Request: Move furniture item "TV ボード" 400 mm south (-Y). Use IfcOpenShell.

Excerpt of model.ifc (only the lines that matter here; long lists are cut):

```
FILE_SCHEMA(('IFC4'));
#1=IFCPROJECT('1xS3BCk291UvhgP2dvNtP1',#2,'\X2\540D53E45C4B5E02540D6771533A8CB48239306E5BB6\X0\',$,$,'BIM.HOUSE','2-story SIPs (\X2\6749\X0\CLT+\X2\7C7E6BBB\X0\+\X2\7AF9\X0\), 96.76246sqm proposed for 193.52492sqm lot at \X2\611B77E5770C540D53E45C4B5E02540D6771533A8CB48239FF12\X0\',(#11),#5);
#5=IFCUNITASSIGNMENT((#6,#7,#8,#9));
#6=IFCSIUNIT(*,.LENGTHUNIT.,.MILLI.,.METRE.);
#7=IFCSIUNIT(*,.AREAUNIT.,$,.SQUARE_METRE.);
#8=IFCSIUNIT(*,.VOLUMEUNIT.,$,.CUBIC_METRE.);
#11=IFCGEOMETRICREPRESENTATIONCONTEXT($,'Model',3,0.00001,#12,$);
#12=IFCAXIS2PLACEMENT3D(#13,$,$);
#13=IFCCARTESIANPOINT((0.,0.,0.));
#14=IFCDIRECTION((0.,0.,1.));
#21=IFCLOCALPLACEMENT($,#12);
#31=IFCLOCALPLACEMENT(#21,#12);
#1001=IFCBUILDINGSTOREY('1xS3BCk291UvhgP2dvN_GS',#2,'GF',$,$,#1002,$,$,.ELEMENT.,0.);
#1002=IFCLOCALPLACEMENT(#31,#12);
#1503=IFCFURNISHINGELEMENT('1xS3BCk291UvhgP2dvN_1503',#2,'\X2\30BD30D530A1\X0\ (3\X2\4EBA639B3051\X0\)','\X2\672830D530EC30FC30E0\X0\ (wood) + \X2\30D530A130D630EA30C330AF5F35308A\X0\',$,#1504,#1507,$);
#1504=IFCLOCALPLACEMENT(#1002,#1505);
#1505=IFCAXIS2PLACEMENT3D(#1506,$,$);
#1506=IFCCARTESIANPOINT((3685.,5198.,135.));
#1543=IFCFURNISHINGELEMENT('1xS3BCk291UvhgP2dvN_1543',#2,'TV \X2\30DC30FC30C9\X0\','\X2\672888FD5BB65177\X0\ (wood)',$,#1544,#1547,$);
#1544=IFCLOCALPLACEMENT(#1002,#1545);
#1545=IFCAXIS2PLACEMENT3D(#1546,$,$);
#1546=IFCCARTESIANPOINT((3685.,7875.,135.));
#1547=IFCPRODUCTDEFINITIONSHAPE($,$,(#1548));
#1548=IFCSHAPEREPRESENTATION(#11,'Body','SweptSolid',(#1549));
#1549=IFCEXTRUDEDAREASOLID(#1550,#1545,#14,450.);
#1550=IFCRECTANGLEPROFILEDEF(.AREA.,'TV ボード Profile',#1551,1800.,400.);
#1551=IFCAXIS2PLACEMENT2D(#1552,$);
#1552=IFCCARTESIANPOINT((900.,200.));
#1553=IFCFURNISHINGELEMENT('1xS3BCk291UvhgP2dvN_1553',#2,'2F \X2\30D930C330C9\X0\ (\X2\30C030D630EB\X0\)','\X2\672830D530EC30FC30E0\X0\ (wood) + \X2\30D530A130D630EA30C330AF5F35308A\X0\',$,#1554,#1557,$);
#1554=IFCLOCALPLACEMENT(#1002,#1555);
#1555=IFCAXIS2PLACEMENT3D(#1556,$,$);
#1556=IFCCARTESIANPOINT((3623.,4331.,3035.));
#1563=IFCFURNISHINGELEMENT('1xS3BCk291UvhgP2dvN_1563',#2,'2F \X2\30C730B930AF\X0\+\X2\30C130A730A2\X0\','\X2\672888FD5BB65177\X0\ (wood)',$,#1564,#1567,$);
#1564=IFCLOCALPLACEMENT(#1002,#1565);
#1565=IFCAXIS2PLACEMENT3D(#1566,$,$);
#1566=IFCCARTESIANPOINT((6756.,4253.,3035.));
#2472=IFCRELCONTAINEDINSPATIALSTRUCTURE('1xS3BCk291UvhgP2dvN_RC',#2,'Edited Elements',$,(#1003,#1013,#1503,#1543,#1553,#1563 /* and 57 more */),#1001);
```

```python
import ifcopenshell
import ifcopenshell.api.geometry
import ifcopenshell.util.placement
import ifcopenshell.util.unit

model = ifcopenshell.open("model.ifc")
unit_scale = ifcopenshell.util.unit.calculate_unit_scale(model)

item = model.by_guid("1xS3BCk291UvhgP2dvN_1543")
matrix = ifcopenshell.util.placement.get_local_placement(item.ObjectPlacement)
matrix[1, 3] -= 0.4 / unit_scale
ifcopenshell.api.geometry.edit_object_placement(model, product=item, matrix=matrix, is_si=False)

print(ifcopenshell.util.placement.get_local_placement(item.ObjectPlacement).round(3) + 0.0)

model.write("model_edited.ifc")
```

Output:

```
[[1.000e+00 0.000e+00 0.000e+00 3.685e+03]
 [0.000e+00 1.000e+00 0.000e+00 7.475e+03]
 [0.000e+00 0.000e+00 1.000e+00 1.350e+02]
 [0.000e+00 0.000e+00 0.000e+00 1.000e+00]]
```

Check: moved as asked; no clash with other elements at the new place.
